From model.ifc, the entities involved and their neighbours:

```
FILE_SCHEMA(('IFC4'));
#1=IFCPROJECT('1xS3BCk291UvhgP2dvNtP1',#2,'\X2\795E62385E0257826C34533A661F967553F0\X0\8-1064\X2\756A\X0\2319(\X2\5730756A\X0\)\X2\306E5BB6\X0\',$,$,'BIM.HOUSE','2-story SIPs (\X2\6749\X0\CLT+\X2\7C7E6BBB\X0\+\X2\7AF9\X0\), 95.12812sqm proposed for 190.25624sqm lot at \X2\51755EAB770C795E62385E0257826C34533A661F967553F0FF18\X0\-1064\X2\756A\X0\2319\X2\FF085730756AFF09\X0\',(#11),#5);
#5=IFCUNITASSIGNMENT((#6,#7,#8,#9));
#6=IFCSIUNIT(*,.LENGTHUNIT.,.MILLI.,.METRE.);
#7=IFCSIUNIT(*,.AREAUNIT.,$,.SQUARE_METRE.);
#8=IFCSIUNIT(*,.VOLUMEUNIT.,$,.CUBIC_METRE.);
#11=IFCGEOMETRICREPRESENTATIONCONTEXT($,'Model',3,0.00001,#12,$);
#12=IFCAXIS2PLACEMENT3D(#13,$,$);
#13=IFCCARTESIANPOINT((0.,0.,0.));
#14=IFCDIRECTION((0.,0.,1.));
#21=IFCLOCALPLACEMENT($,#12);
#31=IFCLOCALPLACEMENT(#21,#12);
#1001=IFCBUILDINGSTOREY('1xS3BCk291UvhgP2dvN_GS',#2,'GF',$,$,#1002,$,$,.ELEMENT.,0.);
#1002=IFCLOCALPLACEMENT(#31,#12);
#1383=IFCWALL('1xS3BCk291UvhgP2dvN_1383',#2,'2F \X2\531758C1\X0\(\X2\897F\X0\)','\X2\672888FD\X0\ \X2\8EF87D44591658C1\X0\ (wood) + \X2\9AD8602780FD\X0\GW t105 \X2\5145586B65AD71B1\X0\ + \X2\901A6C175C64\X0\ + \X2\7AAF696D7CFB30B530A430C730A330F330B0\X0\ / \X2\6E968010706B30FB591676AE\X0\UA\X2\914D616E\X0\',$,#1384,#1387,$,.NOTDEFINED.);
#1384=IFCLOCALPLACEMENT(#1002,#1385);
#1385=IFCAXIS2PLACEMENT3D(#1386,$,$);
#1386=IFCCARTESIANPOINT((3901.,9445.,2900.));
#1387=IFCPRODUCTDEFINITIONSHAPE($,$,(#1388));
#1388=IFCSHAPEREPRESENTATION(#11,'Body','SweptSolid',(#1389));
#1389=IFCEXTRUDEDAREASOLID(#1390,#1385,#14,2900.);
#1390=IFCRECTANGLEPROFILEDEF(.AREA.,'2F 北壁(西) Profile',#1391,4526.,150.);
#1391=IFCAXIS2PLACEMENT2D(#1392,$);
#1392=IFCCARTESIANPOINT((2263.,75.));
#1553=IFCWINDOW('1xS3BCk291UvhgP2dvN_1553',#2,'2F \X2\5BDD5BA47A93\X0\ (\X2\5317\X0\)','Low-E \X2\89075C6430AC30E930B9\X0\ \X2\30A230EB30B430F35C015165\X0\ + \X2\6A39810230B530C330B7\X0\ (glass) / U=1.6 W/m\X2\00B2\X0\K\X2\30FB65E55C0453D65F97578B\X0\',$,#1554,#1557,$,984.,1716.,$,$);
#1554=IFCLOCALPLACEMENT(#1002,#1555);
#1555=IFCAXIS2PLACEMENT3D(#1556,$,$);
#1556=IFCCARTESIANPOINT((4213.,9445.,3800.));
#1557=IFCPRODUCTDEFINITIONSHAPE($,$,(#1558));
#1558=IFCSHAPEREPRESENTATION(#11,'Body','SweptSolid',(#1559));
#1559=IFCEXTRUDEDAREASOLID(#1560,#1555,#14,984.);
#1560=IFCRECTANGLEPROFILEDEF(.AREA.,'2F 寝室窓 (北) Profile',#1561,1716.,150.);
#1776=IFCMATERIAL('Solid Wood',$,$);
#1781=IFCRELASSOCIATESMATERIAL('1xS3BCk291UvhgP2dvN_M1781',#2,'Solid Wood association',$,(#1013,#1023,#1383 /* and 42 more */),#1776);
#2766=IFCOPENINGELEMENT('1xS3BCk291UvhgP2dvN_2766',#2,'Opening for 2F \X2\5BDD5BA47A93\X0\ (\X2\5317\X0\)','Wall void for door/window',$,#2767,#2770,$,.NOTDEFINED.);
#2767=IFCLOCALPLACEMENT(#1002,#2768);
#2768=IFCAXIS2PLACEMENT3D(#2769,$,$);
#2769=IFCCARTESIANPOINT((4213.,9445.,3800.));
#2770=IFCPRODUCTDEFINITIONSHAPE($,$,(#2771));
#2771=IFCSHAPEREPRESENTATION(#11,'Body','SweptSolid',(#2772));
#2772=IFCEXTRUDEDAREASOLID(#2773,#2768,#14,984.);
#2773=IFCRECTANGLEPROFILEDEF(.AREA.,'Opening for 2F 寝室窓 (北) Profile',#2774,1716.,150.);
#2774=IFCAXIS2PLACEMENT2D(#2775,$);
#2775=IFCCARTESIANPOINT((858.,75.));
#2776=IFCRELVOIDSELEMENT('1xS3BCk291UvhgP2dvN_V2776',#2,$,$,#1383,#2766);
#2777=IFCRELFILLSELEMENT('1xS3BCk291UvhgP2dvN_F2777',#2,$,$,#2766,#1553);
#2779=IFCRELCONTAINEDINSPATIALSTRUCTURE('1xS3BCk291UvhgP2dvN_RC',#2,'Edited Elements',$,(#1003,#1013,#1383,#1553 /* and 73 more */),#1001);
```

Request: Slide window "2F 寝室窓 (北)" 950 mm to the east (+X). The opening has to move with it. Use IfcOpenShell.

```python
import ifcopenshell
import ifcopenshell.api.geometry
import ifcopenshell.util.placement
import ifcopenshell.util.unit

model = ifcopenshell.open("model.ifc")
unit_scale = ifcopenshell.util.unit.calculate_unit_scale(model)

window = model.by_guid("1xS3BCk291UvhgP2dvN_1553")
opening = window.FillsVoids[0].RelatingOpeningElement
wall = opening.VoidsElements[0].RelatingBuildingElement

wall_matrix = ifcopenshell.util.placement.get_local_placement(wall.ObjectPlacement)
shift = wall_matrix[:3, 0] * 0.95 / unit_scale
before = ifcopenshell.util.placement.get_local_placement(window.ObjectPlacement)[:3, 3].copy()

# The window is not placed relative to its opening, so move both.
for product in (opening, window):
    matrix = ifcopenshell.util.placement.get_local_placement(product.ObjectPlacement)
    matrix[:3, 3] += shift
    ifcopenshell.api.geometry.edit_object_placement(model, product=product, matrix=matrix, is_si=False)

after = ifcopenshell.util.placement.get_local_placement(window.ObjectPlacement)[:3, 3]
print("window moved by", (after - before).round(3) + 0.0)

model.write("model_updated.ifc")
```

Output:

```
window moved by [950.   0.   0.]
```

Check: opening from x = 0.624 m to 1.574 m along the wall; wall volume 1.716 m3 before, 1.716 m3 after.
